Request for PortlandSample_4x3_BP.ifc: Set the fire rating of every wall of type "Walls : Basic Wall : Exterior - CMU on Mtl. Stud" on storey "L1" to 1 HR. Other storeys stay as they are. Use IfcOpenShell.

First a look at what the model holds.

```python
import ifcopenshell
import ifcopenshell.util.element

model = ifcopenshell.open("PortlandSample_4x3_BP.ifc")
print(model.schema)
storey = next(s for s in model.by_type("IfcBuildingStorey") if s.Name == "L1")
walls = [e for e in ifcopenshell.util.element.get_decomposition(storey) if e.is_a("IfcWall")]
seen = {}
for e in walls:
    element_type = ifcopenshell.util.element.get_type(e)
    key = (element_type.Name if element_type != e and element_type else None, ifcopenshell.util.element.get_pset(e, "Pset_WallCommon", "FireRating"))
    seen[key] = seen.get(key, 0) + 1
for (name, value), count in sorted(seen.items(), key=str):
    print(count, "x", name, "|", value)
```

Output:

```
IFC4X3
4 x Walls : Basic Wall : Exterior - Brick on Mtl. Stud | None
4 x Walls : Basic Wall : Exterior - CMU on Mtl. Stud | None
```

```python
import ifcopenshell
import ifcopenshell.api.pset
import ifcopenshell.util.element

model = ifcopenshell.open("PortlandSample_4x3_BP.ifc")

storey = next(s for s in model.by_type("IfcBuildingStorey") if s.Name == "L1")
walls = [e for e in ifcopenshell.util.element.get_decomposition(storey) if e.is_a("IfcWall")]

count = 0
for e in walls:
    element_type = ifcopenshell.util.element.get_type(e)
    if element_type in (None, e) or element_type.Name != "Walls : Basic Wall : Exterior - CMU on Mtl. Stud":
        continue
    # add_pset returns the element's existing set when there is one.
    pset = ifcopenshell.api.pset.add_pset(model, product=e, name="Pset_WallCommon")
    ifcopenshell.api.pset.edit_pset(model, pset=pset, properties={"FireRating": "1 HR"})
    count += 1

print(count, "walls updated")

model.write("PortlandSample_4x3_BP_updated.ifc")
```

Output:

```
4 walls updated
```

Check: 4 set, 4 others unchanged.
